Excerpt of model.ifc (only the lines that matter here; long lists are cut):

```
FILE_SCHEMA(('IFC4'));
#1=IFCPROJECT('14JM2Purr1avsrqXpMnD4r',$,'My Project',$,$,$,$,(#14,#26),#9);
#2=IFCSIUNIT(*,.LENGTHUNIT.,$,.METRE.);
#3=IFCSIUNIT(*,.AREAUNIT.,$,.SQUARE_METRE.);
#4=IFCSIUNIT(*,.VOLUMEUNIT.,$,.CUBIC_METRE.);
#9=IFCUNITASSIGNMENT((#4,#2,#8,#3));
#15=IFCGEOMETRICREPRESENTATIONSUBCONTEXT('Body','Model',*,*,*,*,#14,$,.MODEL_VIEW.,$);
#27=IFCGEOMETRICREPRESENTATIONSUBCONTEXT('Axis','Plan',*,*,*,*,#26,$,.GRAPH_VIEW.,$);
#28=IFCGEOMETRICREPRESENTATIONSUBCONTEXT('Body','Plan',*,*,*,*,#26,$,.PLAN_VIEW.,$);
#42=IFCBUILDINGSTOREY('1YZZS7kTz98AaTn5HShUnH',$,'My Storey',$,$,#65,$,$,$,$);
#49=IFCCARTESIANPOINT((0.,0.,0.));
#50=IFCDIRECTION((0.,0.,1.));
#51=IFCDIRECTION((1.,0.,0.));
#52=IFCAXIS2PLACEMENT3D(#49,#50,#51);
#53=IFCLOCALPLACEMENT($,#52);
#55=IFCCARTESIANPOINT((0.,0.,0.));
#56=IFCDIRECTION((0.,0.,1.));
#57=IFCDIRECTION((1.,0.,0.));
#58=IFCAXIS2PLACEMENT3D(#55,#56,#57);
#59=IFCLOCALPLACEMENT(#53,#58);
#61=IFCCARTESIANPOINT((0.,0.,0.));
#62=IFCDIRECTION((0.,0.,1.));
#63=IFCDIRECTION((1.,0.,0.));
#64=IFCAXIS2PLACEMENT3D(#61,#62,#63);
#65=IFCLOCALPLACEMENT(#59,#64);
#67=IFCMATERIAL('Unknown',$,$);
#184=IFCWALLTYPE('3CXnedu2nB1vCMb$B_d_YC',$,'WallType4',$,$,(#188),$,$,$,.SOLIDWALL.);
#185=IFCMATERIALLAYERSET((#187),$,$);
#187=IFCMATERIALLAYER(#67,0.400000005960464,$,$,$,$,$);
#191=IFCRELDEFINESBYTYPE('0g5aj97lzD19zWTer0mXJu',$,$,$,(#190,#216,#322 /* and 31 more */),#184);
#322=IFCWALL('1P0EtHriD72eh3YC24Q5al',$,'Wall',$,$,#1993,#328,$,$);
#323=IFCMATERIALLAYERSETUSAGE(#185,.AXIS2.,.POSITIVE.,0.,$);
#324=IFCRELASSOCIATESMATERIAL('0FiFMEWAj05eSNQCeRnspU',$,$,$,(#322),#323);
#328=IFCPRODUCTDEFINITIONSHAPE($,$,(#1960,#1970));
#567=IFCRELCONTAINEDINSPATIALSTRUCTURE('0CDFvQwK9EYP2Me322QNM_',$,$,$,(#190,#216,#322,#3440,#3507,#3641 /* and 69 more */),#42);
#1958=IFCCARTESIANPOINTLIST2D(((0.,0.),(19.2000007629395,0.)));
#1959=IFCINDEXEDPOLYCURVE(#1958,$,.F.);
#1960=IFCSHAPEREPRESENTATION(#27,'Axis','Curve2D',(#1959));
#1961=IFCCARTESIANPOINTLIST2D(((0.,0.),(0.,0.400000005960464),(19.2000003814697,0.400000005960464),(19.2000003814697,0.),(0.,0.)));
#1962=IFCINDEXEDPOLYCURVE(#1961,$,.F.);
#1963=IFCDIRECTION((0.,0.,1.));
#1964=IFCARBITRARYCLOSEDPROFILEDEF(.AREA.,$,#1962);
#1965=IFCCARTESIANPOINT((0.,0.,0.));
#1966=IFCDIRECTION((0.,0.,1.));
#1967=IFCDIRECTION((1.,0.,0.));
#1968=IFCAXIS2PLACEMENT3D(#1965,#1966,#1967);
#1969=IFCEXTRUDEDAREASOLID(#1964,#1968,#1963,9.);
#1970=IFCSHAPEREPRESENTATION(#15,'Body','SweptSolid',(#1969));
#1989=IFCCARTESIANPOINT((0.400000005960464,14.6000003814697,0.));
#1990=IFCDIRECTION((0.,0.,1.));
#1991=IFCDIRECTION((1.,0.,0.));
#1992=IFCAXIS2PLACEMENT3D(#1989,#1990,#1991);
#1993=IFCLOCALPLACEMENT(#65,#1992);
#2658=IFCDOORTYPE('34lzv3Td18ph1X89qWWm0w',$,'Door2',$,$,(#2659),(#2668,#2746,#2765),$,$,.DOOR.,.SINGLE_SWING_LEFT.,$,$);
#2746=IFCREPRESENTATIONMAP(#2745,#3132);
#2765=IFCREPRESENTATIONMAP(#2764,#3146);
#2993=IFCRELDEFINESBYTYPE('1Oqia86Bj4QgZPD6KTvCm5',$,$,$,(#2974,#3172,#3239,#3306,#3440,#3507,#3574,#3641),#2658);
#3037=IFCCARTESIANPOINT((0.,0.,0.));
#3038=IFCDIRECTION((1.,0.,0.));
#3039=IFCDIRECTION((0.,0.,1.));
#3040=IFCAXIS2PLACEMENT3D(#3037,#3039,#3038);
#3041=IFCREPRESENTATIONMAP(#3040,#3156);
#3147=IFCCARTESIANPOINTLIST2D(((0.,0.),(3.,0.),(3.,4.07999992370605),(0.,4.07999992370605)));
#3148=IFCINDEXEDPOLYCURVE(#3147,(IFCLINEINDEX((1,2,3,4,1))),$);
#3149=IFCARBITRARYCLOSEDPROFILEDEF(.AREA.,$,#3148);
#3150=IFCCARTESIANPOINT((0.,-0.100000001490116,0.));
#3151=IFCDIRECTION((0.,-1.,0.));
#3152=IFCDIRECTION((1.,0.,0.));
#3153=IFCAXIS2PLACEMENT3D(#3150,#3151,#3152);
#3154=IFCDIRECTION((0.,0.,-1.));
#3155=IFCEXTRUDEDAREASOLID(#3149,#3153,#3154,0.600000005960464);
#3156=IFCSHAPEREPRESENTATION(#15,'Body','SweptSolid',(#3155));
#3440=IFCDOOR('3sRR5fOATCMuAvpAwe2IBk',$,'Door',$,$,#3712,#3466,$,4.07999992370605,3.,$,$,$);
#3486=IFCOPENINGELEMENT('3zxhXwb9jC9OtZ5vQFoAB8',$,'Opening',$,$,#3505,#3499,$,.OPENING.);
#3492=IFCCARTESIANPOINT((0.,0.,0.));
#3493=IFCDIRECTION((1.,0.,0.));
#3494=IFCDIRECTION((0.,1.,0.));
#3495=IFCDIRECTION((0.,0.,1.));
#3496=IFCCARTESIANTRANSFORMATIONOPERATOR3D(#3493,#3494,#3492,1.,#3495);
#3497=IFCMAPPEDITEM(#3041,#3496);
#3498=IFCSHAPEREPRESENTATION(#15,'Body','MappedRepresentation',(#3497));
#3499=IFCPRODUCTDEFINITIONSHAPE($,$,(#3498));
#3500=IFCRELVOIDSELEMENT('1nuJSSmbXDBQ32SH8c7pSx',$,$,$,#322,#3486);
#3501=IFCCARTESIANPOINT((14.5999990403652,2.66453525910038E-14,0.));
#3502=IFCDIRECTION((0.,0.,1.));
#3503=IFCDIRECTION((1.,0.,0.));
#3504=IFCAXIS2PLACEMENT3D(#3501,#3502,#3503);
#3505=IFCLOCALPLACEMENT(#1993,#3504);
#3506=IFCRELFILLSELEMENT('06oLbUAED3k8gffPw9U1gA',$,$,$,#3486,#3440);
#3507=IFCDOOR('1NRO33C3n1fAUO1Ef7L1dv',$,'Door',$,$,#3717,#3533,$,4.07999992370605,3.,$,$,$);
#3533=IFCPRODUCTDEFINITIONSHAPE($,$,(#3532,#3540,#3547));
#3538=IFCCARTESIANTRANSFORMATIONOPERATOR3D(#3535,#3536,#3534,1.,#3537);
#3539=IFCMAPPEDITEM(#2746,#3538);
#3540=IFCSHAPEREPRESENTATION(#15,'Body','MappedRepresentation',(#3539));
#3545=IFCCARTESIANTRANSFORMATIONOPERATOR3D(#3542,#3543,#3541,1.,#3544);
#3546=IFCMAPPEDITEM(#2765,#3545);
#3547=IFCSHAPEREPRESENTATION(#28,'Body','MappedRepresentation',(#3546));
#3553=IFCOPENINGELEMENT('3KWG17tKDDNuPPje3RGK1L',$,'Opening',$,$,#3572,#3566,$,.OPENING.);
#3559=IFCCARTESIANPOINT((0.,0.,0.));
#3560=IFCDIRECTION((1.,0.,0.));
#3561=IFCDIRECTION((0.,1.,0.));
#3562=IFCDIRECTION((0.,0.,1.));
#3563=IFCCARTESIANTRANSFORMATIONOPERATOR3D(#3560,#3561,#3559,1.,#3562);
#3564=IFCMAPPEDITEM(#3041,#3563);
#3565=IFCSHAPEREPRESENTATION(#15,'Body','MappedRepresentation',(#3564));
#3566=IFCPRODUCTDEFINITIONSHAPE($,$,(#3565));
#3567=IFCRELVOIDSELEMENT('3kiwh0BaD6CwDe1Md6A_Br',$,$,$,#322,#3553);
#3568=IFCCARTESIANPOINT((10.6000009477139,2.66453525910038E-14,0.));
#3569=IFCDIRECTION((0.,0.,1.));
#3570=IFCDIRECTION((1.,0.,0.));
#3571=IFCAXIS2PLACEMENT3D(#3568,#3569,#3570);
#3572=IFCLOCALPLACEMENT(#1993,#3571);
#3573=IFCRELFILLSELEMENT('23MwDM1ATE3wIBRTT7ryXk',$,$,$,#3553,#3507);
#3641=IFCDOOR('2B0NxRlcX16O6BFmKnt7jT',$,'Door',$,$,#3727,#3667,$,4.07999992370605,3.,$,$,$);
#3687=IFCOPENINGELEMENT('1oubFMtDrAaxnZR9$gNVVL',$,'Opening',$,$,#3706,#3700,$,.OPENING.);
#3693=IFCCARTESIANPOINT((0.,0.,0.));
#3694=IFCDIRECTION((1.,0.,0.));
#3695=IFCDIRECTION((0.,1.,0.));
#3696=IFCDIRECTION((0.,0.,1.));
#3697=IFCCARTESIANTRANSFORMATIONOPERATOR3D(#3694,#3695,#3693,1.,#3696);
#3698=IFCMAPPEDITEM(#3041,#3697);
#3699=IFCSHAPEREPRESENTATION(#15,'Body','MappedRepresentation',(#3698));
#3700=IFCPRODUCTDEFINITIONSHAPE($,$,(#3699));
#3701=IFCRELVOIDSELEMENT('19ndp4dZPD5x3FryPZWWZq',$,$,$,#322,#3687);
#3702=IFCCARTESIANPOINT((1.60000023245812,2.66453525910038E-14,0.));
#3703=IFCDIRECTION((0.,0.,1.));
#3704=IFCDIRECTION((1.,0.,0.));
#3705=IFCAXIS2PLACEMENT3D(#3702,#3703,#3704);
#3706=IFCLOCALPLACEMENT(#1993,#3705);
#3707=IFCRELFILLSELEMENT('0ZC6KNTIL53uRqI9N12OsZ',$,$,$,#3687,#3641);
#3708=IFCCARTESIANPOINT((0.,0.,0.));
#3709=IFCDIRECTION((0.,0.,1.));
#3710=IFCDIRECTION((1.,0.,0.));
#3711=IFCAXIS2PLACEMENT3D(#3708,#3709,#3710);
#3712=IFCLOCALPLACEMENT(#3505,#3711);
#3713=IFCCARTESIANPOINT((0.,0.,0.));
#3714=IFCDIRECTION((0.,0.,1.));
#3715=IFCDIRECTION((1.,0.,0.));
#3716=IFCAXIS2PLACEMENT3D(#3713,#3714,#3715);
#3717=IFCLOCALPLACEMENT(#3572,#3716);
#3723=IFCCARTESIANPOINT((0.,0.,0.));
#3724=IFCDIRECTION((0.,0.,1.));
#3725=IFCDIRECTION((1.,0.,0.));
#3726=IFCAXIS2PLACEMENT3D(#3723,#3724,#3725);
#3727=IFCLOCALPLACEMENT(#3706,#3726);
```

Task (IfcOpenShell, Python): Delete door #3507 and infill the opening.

```python
import ifcopenshell
import ifcopenshell.api.feature
import ifcopenshell.api.root
import ifcopenshell.geom
import ifcopenshell.util.shape

model = ifcopenshell.open("model.ifc")
settings = ifcopenshell.geom.settings()


def volume(element):
    """Net volume in cubic metres, openings subtracted."""
    shape = ifcopenshell.geom.create_shape(settings, element)
    return ifcopenshell.util.shape.get_volume(shape.geometry)


door = model.by_guid("1NRO33C3n1fAUO1Ef7L1dv")
opening = door.FillsVoids[0].RelatingOpeningElement
wall = opening.VoidsElements[0].RelatingBuildingElement
before = volume(wall)

ifcopenshell.api.root.remove_product(model, product=door)
ifcopenshell.api.feature.remove_feature(model, feature=opening)

after = volume(wall)

print(f"wall volume {before:.3f} -> {after:.3f} m3")

model.write("model_rev.ifc")
```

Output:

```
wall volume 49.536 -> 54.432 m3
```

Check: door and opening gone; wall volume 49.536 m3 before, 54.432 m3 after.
